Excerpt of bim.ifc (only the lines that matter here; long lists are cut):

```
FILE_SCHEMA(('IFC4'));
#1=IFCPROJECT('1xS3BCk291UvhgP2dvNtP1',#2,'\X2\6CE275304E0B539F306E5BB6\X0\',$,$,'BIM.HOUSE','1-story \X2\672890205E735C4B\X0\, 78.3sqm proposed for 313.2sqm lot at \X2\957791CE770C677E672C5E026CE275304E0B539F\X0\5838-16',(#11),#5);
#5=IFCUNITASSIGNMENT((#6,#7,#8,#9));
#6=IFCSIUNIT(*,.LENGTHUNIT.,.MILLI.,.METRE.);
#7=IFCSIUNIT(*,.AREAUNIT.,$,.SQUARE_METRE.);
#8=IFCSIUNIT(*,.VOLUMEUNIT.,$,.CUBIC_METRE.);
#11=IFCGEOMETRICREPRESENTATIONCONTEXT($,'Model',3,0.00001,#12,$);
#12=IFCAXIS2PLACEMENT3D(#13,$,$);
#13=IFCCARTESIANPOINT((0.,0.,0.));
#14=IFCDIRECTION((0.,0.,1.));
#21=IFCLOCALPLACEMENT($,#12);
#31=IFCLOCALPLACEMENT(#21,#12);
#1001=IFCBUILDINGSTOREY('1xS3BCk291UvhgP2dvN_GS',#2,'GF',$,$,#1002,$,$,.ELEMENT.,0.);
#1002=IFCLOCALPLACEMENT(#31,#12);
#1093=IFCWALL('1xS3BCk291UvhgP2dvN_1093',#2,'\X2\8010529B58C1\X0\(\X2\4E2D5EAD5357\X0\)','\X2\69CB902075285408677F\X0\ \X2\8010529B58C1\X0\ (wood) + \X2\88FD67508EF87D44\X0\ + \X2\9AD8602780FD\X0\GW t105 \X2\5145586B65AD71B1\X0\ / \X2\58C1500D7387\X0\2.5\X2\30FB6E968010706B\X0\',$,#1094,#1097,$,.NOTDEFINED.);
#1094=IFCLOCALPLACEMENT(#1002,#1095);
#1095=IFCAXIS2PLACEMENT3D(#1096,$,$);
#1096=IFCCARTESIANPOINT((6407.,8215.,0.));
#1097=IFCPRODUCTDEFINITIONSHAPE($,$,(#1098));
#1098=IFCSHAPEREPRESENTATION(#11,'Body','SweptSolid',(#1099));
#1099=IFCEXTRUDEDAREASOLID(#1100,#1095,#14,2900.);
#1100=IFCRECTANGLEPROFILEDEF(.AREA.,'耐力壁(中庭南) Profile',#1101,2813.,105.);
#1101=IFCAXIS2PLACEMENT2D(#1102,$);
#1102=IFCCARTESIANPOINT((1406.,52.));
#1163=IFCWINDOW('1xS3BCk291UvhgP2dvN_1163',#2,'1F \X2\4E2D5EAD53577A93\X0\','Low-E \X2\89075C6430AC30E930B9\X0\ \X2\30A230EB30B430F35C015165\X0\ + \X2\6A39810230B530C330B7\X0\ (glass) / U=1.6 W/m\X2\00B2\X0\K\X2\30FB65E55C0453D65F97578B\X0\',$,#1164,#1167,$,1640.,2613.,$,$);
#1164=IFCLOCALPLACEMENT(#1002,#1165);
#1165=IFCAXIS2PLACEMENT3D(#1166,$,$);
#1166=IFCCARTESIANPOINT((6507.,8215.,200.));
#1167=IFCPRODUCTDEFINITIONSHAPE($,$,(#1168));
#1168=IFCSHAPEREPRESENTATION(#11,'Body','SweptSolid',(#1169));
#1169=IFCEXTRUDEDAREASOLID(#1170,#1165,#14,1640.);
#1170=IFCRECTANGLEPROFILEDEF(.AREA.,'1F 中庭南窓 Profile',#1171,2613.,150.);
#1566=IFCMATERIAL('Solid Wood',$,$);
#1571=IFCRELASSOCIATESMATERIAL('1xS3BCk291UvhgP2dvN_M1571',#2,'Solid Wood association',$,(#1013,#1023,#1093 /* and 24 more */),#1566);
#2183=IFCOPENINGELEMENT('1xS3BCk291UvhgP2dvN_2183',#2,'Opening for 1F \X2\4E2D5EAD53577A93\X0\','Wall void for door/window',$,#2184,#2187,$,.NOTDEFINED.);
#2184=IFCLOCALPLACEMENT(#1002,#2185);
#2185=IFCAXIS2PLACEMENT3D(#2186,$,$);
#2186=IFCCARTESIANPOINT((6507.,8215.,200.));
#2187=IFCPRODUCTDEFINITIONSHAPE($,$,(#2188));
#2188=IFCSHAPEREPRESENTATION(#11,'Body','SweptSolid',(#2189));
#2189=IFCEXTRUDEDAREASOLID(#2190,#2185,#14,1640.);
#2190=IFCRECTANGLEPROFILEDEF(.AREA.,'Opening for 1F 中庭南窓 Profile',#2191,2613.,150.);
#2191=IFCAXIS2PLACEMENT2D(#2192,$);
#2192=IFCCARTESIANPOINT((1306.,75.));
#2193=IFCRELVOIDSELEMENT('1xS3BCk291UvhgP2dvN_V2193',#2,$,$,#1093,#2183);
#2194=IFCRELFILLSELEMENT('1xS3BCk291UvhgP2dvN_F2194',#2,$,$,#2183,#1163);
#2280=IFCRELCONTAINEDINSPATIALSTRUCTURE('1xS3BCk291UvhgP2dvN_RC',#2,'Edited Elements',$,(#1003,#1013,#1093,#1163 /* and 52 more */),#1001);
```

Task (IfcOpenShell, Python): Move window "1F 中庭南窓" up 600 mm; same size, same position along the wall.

```python
import numpy as np
import ifcopenshell
import ifcopenshell.api.geometry
import ifcopenshell.util.placement
import ifcopenshell.util.unit

model = ifcopenshell.open("bim.ifc")
unit_scale = ifcopenshell.util.unit.calculate_unit_scale(model)

window = model.by_guid("1xS3BCk291UvhgP2dvN_1163")
opening = window.FillsVoids[0].RelatingOpeningElement
dz = 600.0

shift = np.array([0.0, 0.0, dz])
# The window is not placed relative to its opening, so move both.
for product in (opening, window):
    matrix = ifcopenshell.util.placement.get_local_placement(product.ObjectPlacement)
    matrix[:3, 3] += shift
    ifcopenshell.api.geometry.edit_object_placement(model, product=product, matrix=matrix, is_si=False)

print(f"moved by {dz * unit_scale:+.3f} m")

model.write("bim_edited.ifc")
```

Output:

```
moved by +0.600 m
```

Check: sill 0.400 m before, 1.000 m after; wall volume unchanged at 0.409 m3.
